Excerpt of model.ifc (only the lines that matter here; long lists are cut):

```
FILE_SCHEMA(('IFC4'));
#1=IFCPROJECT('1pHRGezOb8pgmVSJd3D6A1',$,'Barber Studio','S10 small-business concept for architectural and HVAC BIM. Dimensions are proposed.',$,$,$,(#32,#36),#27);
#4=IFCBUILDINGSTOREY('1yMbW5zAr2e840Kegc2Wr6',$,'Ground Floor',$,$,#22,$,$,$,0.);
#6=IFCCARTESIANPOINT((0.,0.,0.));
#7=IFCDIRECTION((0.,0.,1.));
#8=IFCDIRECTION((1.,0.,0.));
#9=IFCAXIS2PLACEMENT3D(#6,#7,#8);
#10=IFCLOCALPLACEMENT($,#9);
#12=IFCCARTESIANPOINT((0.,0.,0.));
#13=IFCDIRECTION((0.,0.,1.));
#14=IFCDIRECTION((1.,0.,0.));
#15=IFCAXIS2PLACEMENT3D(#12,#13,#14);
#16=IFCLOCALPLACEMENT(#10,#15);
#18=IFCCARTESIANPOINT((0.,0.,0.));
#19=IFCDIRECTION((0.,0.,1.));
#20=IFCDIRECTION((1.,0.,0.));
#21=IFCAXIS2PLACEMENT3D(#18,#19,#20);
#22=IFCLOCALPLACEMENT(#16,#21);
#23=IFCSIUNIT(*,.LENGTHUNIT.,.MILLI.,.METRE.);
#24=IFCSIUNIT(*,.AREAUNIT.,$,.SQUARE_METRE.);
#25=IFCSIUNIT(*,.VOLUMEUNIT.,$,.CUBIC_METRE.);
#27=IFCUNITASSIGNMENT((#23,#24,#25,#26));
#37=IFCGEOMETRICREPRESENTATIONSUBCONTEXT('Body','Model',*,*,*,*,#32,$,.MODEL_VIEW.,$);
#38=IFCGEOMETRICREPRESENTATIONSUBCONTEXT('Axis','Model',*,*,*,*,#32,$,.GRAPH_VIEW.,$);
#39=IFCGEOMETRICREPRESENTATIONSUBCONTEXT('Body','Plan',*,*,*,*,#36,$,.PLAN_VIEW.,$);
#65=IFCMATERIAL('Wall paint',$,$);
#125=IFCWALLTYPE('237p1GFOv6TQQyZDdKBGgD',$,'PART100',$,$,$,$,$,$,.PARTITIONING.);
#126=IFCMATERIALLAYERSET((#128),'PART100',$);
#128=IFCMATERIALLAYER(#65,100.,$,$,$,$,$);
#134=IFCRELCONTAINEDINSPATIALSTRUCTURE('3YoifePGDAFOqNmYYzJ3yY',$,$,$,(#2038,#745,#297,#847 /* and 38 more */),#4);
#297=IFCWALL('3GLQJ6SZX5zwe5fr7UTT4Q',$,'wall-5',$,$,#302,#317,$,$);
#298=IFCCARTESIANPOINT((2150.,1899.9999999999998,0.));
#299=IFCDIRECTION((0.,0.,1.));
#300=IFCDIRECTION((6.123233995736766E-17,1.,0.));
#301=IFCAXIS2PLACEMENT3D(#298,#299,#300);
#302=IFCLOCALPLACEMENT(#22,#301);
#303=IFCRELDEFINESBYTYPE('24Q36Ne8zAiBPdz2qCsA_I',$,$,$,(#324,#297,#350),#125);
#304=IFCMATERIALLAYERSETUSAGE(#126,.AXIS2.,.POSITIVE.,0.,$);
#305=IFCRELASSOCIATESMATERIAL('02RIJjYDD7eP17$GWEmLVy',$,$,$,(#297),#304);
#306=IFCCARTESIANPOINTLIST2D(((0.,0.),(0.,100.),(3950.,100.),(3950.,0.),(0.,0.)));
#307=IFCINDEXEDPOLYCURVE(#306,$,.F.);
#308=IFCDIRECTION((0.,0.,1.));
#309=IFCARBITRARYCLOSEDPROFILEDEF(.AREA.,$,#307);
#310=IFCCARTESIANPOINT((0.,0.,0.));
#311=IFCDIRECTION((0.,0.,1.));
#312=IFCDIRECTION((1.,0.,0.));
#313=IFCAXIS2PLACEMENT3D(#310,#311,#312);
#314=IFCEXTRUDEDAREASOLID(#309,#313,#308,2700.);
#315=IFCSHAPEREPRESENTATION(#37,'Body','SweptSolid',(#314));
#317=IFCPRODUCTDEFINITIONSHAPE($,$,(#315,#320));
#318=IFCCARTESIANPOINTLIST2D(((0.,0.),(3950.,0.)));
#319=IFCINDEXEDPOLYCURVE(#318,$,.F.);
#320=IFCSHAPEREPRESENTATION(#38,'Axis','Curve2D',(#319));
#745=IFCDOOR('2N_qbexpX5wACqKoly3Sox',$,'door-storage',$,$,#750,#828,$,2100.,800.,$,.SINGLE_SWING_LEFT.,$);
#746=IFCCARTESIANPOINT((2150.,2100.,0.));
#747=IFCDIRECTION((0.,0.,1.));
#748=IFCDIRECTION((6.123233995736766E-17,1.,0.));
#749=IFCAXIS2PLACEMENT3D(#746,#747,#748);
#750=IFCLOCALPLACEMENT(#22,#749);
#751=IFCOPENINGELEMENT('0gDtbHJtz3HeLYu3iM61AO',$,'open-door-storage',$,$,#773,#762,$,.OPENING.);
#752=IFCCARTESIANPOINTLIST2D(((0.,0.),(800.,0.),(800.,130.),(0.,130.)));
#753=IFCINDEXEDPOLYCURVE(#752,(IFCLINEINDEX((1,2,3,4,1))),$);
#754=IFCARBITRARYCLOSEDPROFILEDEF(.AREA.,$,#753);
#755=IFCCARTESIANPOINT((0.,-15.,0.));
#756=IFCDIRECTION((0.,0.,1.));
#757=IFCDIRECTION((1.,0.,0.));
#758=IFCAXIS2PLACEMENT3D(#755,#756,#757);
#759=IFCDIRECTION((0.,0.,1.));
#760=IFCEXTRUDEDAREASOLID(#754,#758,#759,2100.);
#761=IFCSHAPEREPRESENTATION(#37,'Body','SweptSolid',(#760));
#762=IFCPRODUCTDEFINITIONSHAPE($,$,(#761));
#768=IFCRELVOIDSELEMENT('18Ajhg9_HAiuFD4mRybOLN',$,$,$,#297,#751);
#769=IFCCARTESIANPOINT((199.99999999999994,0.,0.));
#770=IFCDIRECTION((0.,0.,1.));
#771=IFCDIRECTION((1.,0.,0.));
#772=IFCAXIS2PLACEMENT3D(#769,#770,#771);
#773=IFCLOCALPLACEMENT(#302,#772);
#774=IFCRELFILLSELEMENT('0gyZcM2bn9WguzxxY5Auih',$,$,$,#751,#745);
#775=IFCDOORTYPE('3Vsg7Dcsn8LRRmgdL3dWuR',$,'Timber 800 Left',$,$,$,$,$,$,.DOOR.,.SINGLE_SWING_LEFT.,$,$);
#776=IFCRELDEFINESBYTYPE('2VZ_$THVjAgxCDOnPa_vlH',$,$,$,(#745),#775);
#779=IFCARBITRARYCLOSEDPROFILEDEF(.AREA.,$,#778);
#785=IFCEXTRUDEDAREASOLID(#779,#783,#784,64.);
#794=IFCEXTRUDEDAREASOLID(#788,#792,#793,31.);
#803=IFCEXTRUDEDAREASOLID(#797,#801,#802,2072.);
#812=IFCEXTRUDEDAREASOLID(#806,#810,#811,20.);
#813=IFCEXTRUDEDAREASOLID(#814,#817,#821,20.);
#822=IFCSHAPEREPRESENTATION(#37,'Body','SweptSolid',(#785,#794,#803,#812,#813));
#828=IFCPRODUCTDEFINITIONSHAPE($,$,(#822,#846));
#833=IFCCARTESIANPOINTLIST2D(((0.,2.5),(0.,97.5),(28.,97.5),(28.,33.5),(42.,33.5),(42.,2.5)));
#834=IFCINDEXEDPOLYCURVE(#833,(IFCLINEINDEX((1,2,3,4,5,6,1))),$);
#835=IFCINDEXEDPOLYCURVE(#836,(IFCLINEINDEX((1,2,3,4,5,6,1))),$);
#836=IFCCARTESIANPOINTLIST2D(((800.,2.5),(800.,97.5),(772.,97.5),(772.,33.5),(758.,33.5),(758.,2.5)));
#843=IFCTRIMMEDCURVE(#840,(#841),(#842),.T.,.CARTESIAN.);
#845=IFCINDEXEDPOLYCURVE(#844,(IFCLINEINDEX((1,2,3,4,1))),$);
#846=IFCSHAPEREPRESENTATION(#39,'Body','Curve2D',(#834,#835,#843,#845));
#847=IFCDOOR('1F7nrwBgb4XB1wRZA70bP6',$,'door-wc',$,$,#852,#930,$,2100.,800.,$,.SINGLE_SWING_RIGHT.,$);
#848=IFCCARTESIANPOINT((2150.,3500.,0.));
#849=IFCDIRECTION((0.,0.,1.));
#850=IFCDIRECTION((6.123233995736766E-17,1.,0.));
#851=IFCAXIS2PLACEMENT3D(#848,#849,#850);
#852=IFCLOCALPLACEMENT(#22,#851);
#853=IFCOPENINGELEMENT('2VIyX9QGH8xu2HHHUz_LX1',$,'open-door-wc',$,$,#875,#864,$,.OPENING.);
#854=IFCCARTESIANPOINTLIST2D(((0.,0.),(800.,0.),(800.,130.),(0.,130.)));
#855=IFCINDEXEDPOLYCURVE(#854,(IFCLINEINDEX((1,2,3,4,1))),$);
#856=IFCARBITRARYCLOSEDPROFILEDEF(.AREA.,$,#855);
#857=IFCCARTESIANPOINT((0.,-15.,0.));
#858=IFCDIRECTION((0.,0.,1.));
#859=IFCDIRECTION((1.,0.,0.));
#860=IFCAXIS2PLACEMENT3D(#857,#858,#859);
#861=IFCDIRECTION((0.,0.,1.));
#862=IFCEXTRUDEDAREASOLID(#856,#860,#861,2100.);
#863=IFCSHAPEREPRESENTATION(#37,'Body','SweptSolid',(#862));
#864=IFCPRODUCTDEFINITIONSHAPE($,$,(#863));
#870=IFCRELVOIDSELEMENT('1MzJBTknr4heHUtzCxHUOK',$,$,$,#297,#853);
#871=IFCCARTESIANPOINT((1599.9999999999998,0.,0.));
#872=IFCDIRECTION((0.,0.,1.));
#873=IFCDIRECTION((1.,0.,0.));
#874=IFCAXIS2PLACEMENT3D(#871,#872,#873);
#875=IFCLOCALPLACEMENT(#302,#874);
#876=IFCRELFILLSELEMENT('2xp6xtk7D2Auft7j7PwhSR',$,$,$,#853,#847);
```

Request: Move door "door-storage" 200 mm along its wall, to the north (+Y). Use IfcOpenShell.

```python
import ifcopenshell
import ifcopenshell.api.geometry
import ifcopenshell.util.placement

model = ifcopenshell.open("model.ifc")

door = model.by_id(745)
opening = door.FillsVoids[0].RelatingOpeningElement
wall = opening.VoidsElements[0].RelatingBuildingElement

wall_matrix = ifcopenshell.util.placement.get_local_placement(wall.ObjectPlacement)
shift = wall_matrix[:3, 0] * 200.0
before = ifcopenshell.util.placement.get_local_placement(door.ObjectPlacement)[:3, 3].copy()

# The door is not placed relative to its opening, so move both.
for product in (opening, door):
    matrix = ifcopenshell.util.placement.get_local_placement(product.ObjectPlacement)
    matrix[:3, 3] += shift
    ifcopenshell.api.geometry.edit_object_placement(model, product=product, matrix=matrix, is_si=False)

after = ifcopenshell.util.placement.get_local_placement(door.ObjectPlacement)[:3, 3]
print("door moved by", (after - before).round(3) + 0.0)

model.write("model-out.ifc")
```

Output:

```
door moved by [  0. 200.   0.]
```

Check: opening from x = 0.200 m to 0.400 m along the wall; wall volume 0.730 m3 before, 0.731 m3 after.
